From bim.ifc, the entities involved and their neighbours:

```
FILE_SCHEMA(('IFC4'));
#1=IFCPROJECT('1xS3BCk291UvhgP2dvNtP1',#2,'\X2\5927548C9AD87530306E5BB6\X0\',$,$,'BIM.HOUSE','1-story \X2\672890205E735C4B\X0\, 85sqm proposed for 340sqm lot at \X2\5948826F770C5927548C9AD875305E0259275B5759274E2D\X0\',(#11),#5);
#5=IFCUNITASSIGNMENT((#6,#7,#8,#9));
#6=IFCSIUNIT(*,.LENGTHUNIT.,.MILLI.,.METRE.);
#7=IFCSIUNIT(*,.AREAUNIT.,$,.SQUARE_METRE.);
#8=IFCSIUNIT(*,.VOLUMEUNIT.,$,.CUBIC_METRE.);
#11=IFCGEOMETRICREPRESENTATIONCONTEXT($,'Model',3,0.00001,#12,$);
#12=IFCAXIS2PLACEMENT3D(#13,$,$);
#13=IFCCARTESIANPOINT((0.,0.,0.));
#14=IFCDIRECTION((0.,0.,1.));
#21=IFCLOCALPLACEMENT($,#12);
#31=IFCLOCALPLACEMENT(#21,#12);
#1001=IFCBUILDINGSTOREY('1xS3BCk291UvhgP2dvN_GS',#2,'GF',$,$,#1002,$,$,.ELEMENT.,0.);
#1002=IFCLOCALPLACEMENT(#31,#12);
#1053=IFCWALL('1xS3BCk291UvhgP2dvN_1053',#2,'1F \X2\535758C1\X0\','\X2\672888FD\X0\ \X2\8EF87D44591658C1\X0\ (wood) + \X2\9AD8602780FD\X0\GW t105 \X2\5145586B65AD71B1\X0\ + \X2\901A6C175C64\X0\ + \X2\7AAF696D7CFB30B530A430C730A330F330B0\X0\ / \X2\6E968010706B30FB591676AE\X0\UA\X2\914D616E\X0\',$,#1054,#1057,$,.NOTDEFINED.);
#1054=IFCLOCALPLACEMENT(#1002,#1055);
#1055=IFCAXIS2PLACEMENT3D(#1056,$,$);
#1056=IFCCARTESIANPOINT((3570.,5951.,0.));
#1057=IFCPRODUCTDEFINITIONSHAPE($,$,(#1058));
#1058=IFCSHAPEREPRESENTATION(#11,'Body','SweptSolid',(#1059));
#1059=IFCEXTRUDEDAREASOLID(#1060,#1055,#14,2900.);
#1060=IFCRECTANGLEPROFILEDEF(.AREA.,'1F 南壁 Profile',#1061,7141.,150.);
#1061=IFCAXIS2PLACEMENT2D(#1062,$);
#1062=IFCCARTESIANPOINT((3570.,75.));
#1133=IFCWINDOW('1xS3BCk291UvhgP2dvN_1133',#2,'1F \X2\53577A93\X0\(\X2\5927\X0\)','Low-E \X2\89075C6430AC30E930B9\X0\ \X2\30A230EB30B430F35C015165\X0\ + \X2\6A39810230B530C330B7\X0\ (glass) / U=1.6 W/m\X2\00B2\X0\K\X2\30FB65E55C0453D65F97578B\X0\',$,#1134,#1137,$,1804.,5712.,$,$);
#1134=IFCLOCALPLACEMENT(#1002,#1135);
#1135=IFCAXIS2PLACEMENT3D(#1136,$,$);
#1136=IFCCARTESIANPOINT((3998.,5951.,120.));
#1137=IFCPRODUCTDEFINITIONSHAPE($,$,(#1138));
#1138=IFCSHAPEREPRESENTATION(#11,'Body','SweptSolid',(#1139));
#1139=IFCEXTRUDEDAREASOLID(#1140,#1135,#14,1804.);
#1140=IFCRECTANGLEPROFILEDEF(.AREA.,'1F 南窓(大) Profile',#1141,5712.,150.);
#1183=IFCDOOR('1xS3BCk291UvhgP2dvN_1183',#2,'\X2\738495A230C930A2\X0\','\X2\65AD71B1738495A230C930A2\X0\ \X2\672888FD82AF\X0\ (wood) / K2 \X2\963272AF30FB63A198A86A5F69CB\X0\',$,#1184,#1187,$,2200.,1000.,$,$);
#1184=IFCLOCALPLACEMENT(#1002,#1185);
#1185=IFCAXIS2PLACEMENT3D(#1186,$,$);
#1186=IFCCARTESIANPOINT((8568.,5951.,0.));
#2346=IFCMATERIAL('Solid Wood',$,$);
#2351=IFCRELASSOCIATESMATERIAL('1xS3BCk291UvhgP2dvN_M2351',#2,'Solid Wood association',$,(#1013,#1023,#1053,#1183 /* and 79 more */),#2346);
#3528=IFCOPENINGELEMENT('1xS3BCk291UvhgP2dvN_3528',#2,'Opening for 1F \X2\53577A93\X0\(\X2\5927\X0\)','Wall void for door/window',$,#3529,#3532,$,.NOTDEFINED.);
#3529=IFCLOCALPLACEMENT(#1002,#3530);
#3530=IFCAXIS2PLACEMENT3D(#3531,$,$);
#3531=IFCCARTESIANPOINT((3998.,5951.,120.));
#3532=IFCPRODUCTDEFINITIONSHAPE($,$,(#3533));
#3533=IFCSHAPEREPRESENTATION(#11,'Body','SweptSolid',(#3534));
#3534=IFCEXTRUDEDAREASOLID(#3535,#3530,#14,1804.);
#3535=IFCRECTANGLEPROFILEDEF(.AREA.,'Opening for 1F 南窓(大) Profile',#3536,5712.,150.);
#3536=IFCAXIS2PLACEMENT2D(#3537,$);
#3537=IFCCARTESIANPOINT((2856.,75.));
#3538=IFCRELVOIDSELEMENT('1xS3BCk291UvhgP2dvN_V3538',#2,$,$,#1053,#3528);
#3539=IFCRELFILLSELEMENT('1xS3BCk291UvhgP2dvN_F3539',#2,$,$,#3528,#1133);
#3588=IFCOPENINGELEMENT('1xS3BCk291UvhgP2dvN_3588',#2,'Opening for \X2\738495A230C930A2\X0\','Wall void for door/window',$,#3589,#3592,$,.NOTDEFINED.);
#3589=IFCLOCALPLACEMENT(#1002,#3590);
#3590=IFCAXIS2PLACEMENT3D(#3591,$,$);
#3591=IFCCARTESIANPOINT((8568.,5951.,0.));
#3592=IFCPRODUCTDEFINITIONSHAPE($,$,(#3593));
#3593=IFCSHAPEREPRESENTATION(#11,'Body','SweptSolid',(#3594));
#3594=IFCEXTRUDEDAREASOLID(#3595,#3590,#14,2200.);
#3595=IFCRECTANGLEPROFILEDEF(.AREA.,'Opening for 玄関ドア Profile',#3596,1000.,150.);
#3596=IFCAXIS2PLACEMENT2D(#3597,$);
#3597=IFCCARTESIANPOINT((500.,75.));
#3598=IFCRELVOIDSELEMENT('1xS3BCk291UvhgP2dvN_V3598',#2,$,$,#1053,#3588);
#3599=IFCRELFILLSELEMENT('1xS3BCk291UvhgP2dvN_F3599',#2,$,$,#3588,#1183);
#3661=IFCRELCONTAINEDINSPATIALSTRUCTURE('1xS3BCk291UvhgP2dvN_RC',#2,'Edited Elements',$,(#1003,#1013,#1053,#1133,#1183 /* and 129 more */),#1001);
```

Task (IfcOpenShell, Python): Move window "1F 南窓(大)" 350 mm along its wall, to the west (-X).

```python
import ifcopenshell
import ifcopenshell.api.geometry
import ifcopenshell.util.placement
import ifcopenshell.util.unit

model = ifcopenshell.open("bim.ifc")
unit_scale = ifcopenshell.util.unit.calculate_unit_scale(model)

window = model.by_id(1133)
opening = window.FillsVoids[0].RelatingOpeningElement
wall = opening.VoidsElements[0].RelatingBuildingElement

wall_matrix = ifcopenshell.util.placement.get_local_placement(wall.ObjectPlacement)
shift = wall_matrix[:3, 0] * -0.35 / unit_scale
before = ifcopenshell.util.placement.get_local_placement(window.ObjectPlacement)[:3, 3].copy()

# The window is not placed relative to its opening, so move both.
for product in (opening, window):
    matrix = ifcopenshell.util.placement.get_local_placement(product.ObjectPlacement)
    matrix[:3, 3] += shift
    ifcopenshell.api.geometry.edit_object_placement(model, product=product, matrix=matrix, is_si=False)

after = ifcopenshell.util.placement.get_local_placement(window.ObjectPlacement)[:3, 3]
print("window moved by", (after - before).round(3) + 0.0)

model.write("bim_edited.ifc")
```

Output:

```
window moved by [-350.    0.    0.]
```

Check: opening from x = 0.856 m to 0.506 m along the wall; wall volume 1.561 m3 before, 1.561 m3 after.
